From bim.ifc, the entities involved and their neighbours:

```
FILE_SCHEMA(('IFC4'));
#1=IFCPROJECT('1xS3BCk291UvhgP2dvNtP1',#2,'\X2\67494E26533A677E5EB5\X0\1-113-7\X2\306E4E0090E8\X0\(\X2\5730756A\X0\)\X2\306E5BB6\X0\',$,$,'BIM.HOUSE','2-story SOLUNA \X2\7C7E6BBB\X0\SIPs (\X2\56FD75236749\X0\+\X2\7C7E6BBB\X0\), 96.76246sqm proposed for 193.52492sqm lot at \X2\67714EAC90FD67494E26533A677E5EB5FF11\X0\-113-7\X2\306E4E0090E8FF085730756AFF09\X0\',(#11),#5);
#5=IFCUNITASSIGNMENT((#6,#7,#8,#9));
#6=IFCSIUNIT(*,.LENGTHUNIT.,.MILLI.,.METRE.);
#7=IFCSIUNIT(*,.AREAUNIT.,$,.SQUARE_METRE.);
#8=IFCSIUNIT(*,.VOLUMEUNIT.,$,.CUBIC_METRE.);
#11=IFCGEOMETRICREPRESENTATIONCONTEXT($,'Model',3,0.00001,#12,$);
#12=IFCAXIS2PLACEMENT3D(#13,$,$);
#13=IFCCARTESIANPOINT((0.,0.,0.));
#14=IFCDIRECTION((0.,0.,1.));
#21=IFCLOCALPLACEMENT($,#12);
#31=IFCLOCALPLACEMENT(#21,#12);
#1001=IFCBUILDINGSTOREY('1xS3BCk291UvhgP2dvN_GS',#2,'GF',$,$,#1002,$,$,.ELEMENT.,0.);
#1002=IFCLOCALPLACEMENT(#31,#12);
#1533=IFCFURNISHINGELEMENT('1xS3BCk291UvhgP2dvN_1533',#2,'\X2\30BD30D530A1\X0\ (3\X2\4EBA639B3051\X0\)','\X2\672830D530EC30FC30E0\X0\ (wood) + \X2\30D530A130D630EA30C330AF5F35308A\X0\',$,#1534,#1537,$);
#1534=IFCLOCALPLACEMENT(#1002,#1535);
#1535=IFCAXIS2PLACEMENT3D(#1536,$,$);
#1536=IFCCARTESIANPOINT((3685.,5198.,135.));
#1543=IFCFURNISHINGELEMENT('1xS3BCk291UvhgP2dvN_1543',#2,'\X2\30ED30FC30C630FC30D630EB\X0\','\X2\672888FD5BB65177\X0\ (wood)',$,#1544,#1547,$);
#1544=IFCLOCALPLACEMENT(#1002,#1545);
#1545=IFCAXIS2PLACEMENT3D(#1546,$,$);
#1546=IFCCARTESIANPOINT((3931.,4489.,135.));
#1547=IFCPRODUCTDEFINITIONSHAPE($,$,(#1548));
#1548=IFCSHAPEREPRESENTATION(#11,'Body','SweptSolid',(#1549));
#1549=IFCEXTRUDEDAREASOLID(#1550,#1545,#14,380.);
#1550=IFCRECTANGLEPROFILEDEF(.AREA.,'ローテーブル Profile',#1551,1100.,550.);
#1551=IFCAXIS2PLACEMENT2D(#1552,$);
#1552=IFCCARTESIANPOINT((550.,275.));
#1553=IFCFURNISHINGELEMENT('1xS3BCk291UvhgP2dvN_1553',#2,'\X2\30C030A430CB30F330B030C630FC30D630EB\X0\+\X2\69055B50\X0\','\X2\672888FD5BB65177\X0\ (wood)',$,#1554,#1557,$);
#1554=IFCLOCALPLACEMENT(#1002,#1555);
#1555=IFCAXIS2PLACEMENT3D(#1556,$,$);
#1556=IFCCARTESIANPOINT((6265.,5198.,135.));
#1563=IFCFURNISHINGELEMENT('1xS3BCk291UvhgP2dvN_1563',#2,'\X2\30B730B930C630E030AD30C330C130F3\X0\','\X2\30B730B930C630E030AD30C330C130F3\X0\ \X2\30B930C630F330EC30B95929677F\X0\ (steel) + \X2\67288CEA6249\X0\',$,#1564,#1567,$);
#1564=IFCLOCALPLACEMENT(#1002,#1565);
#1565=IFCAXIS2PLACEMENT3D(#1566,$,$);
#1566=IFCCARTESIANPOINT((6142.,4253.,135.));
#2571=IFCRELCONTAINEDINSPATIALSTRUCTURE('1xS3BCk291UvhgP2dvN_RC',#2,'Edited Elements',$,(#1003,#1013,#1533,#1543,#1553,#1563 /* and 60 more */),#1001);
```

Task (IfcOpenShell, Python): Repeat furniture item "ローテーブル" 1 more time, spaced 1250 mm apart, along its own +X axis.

```python
import ifcopenshell
import ifcopenshell.api.geometry
import ifcopenshell.api.root
import ifcopenshell.util.element
import ifcopenshell.util.placement
import ifcopenshell.util.unit

model = ifcopenshell.open("bim.ifc")
unit_scale = ifcopenshell.util.unit.calculate_unit_scale(model)


def reuse_history(source, copy):
    """copy_class also copies each property set's owner history, people and application; keep the originals."""
    for rel in copy.IsDefinedBy:
        if rel.is_a("IfcRelDefinesByProperties") and (history := rel.RelatingPropertyDefinition.OwnerHistory):
            rel.RelatingPropertyDefinition.OwnerHistory = source.OwnerHistory
            ifcopenshell.util.element.remove_deep2(model, history)


source = model.by_id(1543)
base = ifcopenshell.util.placement.get_local_placement(source.ObjectPlacement)
step = base[:3, 0] * 1.25 / unit_scale

for i in range(1, 2):
    copy = ifcopenshell.api.root.copy_class(model, product=source)
    copy.Representation = ifcopenshell.util.element.copy_deep(
        model, source.Representation, exclude=["IfcGeometricRepresentationContext", "IfcRepresentationMap"]
    )
    reuse_history(source, copy)
    matrix = base.copy()
    matrix[:3, 3] += i * step
    print("added at", matrix[:3, 3].round(3) + 0.0)
    ifcopenshell.api.geometry.edit_object_placement(model, product=copy, matrix=matrix, is_si=False)

model.write("bim-out.ifc")
```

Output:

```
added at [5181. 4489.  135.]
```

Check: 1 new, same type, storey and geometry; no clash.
